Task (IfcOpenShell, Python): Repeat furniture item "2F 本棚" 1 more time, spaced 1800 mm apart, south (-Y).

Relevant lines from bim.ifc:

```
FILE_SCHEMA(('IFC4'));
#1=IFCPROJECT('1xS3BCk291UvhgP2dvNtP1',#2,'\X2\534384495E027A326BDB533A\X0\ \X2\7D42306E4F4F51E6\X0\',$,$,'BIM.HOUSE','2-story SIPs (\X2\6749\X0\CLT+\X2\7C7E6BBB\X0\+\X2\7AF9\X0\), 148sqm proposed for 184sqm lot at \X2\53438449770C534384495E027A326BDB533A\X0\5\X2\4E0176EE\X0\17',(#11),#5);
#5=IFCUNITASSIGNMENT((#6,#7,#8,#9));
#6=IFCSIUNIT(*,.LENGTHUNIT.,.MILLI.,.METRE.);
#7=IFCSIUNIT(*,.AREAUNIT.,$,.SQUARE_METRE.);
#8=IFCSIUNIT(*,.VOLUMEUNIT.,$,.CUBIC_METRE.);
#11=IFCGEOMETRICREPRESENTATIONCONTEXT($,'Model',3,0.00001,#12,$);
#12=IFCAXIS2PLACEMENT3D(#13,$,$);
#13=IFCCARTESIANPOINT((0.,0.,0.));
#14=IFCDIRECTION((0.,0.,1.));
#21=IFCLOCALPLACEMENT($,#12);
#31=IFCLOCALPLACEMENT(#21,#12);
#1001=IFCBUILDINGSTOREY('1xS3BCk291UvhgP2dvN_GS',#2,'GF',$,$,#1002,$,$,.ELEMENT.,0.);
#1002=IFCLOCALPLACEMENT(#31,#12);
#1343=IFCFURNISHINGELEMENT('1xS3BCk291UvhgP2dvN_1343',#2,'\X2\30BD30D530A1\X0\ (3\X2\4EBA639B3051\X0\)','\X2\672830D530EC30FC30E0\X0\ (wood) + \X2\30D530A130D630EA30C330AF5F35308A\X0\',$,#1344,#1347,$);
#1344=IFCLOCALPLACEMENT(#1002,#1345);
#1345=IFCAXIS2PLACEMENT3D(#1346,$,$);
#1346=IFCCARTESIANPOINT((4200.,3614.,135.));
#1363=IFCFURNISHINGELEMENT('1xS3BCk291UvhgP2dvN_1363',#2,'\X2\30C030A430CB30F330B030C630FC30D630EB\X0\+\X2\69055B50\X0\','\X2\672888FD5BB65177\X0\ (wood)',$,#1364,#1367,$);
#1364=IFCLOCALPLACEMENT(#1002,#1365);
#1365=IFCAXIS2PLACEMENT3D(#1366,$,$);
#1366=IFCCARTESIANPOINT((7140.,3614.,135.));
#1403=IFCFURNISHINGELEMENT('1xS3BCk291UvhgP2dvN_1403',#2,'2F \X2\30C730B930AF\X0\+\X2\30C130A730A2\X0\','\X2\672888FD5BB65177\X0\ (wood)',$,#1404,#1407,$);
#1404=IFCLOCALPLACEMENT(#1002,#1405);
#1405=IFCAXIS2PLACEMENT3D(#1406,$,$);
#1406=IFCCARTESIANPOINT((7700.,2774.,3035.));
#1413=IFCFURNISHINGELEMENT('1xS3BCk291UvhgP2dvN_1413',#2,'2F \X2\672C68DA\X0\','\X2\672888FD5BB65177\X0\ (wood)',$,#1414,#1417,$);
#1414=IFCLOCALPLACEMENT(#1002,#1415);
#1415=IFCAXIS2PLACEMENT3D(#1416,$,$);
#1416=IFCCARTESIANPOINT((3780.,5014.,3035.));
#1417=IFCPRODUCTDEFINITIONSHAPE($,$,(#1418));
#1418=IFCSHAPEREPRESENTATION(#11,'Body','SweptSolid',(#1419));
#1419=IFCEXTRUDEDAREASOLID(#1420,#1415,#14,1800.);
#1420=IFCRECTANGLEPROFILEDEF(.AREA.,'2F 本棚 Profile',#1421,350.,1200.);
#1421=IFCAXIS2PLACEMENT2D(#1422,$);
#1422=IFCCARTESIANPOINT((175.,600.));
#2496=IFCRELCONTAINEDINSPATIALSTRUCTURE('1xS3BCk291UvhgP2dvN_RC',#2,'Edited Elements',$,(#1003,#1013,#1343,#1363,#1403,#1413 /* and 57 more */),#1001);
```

```python
import numpy as np
import ifcopenshell
import ifcopenshell.api.geometry
import ifcopenshell.api.root
import ifcopenshell.util.element
import ifcopenshell.util.placement
import ifcopenshell.util.unit

model = ifcopenshell.open("bim.ifc")
unit_scale = ifcopenshell.util.unit.calculate_unit_scale(model)


def reuse_history(source, copy):
    """copy_class also copies each property set's owner history, people and application; keep the originals."""
    for rel in copy.IsDefinedBy:
        if rel.is_a("IfcRelDefinesByProperties") and (history := rel.RelatingPropertyDefinition.OwnerHistory):
            rel.RelatingPropertyDefinition.OwnerHistory = source.OwnerHistory
            ifcopenshell.util.element.remove_deep2(model, history)


source = model.by_guid("1xS3BCk291UvhgP2dvN_1413")
base = ifcopenshell.util.placement.get_local_placement(source.ObjectPlacement)
step = np.array([0.0, -1.0, 0.0]) * 1.8 / unit_scale

for i in range(1, 2):
    copy = ifcopenshell.api.root.copy_class(model, product=source)
    copy.Representation = ifcopenshell.util.element.copy_deep(
        model, source.Representation, exclude=["IfcGeometricRepresentationContext", "IfcRepresentationMap"]
    )
    reuse_history(source, copy)
    matrix = base.copy()
    matrix[:3, 3] += i * step
    print("added at", matrix[:3, 3].round(3) + 0.0)
    ifcopenshell.api.geometry.edit_object_placement(model, product=copy, matrix=matrix, is_si=False)

model.write("bim_updated.ifc")
```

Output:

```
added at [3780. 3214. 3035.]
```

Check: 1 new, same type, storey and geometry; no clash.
